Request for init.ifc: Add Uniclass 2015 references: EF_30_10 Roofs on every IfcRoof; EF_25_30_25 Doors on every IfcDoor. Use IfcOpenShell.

First a look at what the model holds.

```python
import ifcopenshell

model = ifcopenshell.open("init.ifc")
print(model.schema)
print("classifications:", [c.Name for c in model.by_type("IfcClassification")])
for ifc_class in ("IfcDoor", "IfcRoof", "IfcStair", "IfcWall", "IfcWindow"):
    print(ifc_class, len(model.by_type(ifc_class)))
```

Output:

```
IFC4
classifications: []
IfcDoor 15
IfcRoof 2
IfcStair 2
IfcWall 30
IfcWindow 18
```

```python
import ifcopenshell
import ifcopenshell.api.classification

model = ifcopenshell.open("init.ifc")

system = ifcopenshell.api.classification.add_classification(model, classification="Uniclass 2015")

codes = {
    "IfcRoof": ("EF_30_10", "Roofs"),
    "IfcDoor": ("EF_25_30_25", "Doors"),
}
for ifc_class, (code, name) in codes.items():
    products = model.by_type(ifc_class)
    ifcopenshell.api.classification.add_reference(
        model, products=products, classification=system, identification=code, name=name
    )
    print(code, len(products))

model.write("init_updated.ifc")
```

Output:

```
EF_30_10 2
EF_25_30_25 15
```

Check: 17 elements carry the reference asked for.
